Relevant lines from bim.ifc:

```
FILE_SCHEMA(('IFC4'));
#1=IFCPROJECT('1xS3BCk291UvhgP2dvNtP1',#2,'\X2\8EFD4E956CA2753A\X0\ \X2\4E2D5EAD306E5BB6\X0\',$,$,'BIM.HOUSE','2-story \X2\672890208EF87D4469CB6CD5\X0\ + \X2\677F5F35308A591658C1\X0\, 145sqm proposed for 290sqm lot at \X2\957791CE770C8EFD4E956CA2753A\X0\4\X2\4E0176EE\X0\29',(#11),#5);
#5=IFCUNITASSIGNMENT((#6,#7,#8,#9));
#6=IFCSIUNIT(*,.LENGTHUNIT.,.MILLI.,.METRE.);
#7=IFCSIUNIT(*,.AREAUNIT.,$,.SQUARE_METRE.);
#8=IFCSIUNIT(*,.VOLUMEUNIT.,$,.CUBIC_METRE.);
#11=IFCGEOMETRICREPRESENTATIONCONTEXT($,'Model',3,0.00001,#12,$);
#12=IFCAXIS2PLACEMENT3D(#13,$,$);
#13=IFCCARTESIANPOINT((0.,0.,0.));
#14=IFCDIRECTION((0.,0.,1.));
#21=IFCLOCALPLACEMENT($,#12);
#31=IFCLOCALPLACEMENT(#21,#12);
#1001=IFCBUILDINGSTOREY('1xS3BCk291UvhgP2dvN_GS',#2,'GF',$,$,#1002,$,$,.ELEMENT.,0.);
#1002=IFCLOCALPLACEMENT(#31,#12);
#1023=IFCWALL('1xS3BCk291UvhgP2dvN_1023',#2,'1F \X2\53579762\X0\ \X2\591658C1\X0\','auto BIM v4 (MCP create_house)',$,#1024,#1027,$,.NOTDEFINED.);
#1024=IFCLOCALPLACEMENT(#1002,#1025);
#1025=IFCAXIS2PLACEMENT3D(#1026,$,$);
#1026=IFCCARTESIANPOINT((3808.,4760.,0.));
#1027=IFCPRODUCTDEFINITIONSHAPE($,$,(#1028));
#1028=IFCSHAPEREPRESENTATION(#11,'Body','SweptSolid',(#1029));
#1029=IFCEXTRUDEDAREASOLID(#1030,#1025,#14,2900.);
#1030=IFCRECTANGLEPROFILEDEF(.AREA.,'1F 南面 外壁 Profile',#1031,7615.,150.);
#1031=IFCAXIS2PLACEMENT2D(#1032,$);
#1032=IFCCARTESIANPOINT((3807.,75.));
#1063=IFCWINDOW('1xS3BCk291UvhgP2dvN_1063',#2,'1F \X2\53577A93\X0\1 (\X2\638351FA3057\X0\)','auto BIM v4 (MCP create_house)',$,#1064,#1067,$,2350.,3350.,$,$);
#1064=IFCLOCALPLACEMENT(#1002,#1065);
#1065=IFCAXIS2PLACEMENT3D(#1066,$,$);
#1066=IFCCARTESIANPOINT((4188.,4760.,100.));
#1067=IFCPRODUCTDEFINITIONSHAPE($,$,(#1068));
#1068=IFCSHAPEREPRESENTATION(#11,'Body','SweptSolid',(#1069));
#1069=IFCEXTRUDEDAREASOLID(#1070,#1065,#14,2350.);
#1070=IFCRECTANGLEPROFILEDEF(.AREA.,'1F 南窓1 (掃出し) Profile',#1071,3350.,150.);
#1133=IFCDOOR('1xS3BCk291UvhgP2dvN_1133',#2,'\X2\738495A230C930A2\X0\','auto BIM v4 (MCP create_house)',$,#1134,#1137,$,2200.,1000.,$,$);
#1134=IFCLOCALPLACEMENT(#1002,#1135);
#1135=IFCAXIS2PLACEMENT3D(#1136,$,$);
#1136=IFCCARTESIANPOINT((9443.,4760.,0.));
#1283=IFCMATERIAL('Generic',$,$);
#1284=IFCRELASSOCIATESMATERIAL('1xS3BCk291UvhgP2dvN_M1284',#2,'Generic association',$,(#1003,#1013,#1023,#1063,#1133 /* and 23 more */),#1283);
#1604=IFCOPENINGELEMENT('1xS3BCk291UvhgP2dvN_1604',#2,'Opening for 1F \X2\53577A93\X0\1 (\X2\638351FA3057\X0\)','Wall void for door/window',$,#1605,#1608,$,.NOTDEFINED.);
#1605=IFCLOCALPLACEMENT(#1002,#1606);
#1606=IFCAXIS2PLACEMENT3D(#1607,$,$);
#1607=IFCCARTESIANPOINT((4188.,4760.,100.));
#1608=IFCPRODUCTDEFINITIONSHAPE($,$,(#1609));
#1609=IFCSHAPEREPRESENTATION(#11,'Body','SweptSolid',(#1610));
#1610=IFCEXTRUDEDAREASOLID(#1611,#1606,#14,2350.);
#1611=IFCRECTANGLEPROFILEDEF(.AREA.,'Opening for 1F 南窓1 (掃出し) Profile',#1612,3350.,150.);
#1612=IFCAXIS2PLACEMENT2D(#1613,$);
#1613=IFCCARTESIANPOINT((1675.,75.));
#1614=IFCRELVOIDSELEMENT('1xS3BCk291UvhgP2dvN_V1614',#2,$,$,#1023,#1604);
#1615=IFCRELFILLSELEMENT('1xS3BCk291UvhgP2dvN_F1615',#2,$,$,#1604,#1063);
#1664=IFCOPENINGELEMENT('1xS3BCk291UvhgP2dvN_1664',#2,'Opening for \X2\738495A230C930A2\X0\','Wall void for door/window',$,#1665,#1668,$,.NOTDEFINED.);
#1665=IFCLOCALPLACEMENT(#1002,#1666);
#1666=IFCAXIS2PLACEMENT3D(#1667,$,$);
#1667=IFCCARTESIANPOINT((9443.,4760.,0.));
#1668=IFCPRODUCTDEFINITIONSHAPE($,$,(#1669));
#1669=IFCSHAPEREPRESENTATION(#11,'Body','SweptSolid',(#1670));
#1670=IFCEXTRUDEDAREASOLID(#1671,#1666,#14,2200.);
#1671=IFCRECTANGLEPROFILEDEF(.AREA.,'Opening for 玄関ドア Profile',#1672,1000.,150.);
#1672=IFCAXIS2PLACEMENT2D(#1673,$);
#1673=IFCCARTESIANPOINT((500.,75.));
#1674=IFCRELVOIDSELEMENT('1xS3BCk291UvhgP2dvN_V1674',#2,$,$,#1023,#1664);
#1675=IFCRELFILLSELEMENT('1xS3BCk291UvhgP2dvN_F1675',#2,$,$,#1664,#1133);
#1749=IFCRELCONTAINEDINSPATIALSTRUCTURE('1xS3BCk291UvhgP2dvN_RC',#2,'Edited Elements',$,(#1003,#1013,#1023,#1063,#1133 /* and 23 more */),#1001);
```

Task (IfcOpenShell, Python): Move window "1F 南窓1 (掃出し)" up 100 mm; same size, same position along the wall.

```python
import numpy as np
import ifcopenshell
import ifcopenshell.api.geometry
import ifcopenshell.util.placement
import ifcopenshell.util.unit

model = ifcopenshell.open("bim.ifc")
unit_scale = ifcopenshell.util.unit.calculate_unit_scale(model)

window = model.by_guid("1xS3BCk291UvhgP2dvN_1063")
opening = window.FillsVoids[0].RelatingOpeningElement
dz = 0.1 / unit_scale

shift = np.array([0.0, 0.0, dz])
# The window is not placed relative to its opening, so move both.
for product in (opening, window):
    matrix = ifcopenshell.util.placement.get_local_placement(product.ObjectPlacement)
    matrix[:3, 3] += shift
    ifcopenshell.api.geometry.edit_object_placement(model, product=product, matrix=matrix, is_si=False)

print(f"moved by {dz * unit_scale:+.3f} m")

model.write("bim_v2.ifc")
```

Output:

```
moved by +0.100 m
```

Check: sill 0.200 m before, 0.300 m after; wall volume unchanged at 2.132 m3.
